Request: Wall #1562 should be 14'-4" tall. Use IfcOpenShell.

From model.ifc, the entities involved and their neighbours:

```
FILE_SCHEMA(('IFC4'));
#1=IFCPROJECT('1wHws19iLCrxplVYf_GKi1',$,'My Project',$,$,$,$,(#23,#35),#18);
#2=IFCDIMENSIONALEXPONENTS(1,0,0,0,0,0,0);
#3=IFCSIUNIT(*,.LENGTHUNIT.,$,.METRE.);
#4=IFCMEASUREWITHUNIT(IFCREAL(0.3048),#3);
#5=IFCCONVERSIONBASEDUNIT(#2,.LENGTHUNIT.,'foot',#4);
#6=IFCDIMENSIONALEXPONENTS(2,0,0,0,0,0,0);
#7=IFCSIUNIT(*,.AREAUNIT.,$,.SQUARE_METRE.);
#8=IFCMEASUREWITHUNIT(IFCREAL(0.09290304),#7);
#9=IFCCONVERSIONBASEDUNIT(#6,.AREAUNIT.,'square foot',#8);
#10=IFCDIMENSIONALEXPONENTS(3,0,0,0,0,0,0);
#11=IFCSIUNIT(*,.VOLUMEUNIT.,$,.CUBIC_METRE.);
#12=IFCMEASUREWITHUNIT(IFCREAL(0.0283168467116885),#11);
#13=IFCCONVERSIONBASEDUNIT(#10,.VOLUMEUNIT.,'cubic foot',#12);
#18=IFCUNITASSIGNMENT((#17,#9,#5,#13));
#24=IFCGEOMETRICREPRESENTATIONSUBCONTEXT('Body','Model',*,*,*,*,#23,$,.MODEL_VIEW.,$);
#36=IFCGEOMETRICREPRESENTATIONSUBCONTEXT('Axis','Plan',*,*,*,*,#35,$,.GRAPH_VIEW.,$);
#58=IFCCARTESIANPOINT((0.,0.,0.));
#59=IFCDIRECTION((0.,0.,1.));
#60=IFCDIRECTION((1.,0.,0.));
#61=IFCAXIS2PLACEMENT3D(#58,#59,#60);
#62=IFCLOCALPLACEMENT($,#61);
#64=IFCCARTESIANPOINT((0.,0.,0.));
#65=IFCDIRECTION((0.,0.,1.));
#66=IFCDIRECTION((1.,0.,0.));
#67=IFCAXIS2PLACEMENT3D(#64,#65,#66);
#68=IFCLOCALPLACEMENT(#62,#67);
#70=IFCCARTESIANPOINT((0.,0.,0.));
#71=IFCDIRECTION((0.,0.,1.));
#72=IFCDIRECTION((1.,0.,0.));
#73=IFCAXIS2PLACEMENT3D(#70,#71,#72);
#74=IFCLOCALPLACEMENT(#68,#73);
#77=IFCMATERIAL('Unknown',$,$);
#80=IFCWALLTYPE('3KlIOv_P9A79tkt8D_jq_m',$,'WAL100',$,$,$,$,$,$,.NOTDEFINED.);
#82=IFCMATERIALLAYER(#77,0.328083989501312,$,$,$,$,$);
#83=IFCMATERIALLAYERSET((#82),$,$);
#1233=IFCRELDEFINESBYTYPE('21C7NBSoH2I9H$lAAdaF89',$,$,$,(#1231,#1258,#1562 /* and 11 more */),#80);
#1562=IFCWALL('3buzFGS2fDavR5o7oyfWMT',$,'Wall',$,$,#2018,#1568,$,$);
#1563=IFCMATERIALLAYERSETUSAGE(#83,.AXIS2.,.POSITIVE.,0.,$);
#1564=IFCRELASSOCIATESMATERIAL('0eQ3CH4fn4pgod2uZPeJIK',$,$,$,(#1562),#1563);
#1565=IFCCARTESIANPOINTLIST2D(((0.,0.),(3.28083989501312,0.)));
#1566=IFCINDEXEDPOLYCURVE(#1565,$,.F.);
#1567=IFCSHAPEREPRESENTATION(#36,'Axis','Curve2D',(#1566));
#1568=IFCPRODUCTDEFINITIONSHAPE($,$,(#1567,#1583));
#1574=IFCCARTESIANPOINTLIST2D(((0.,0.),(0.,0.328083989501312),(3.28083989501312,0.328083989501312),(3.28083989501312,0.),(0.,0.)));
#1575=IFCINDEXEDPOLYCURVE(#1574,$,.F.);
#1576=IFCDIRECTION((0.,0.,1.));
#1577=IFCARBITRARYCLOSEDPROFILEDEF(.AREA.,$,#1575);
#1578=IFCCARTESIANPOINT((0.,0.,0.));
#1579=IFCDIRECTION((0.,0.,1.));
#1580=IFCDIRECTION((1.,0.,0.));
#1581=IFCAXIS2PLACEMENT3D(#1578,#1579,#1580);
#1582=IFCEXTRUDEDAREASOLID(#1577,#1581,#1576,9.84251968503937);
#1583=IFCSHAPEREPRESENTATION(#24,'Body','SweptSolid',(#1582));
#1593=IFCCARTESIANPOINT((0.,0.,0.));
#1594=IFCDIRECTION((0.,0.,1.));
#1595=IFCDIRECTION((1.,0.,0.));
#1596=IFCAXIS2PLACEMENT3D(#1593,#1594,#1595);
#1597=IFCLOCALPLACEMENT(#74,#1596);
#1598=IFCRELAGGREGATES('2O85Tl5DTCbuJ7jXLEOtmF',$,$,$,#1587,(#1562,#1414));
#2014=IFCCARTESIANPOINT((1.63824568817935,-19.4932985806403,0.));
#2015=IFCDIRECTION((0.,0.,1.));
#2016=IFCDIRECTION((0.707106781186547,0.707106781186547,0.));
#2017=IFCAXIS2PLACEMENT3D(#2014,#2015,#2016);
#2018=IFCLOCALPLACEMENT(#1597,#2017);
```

```python
import ifcopenshell
import ifcopenshell.geom
import ifcopenshell.util.representation
import ifcopenshell.util.shape
import ifcopenshell.util.unit

model = ifcopenshell.open("model.ifc")
unit_scale = ifcopenshell.util.unit.calculate_unit_scale(model)
settings = ifcopenshell.geom.settings()


def volume(element):
    """Net volume in cubic metres, openings subtracted."""
    shape = ifcopenshell.geom.create_shape(settings, element)
    return ifcopenshell.util.shape.get_volume(shape.geometry)


wall = model.by_guid("3buzFGS2fDavR5o7oyfWMT")
before = volume(wall)

body = ifcopenshell.util.representation.get_representation(wall, "Model", "Body")
solid = body.Items[0]
old_height = solid.Depth
solid.Depth = 172 * 0.0254 / unit_scale
after = volume(wall)

print(f"height {old_height:g} -> {solid.Depth:g}, volume {before:.3f} -> {after:.3f} m3")

model.write("model_updated.ifc")
```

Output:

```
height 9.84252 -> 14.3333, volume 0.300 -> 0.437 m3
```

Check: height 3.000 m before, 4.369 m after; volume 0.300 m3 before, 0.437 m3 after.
